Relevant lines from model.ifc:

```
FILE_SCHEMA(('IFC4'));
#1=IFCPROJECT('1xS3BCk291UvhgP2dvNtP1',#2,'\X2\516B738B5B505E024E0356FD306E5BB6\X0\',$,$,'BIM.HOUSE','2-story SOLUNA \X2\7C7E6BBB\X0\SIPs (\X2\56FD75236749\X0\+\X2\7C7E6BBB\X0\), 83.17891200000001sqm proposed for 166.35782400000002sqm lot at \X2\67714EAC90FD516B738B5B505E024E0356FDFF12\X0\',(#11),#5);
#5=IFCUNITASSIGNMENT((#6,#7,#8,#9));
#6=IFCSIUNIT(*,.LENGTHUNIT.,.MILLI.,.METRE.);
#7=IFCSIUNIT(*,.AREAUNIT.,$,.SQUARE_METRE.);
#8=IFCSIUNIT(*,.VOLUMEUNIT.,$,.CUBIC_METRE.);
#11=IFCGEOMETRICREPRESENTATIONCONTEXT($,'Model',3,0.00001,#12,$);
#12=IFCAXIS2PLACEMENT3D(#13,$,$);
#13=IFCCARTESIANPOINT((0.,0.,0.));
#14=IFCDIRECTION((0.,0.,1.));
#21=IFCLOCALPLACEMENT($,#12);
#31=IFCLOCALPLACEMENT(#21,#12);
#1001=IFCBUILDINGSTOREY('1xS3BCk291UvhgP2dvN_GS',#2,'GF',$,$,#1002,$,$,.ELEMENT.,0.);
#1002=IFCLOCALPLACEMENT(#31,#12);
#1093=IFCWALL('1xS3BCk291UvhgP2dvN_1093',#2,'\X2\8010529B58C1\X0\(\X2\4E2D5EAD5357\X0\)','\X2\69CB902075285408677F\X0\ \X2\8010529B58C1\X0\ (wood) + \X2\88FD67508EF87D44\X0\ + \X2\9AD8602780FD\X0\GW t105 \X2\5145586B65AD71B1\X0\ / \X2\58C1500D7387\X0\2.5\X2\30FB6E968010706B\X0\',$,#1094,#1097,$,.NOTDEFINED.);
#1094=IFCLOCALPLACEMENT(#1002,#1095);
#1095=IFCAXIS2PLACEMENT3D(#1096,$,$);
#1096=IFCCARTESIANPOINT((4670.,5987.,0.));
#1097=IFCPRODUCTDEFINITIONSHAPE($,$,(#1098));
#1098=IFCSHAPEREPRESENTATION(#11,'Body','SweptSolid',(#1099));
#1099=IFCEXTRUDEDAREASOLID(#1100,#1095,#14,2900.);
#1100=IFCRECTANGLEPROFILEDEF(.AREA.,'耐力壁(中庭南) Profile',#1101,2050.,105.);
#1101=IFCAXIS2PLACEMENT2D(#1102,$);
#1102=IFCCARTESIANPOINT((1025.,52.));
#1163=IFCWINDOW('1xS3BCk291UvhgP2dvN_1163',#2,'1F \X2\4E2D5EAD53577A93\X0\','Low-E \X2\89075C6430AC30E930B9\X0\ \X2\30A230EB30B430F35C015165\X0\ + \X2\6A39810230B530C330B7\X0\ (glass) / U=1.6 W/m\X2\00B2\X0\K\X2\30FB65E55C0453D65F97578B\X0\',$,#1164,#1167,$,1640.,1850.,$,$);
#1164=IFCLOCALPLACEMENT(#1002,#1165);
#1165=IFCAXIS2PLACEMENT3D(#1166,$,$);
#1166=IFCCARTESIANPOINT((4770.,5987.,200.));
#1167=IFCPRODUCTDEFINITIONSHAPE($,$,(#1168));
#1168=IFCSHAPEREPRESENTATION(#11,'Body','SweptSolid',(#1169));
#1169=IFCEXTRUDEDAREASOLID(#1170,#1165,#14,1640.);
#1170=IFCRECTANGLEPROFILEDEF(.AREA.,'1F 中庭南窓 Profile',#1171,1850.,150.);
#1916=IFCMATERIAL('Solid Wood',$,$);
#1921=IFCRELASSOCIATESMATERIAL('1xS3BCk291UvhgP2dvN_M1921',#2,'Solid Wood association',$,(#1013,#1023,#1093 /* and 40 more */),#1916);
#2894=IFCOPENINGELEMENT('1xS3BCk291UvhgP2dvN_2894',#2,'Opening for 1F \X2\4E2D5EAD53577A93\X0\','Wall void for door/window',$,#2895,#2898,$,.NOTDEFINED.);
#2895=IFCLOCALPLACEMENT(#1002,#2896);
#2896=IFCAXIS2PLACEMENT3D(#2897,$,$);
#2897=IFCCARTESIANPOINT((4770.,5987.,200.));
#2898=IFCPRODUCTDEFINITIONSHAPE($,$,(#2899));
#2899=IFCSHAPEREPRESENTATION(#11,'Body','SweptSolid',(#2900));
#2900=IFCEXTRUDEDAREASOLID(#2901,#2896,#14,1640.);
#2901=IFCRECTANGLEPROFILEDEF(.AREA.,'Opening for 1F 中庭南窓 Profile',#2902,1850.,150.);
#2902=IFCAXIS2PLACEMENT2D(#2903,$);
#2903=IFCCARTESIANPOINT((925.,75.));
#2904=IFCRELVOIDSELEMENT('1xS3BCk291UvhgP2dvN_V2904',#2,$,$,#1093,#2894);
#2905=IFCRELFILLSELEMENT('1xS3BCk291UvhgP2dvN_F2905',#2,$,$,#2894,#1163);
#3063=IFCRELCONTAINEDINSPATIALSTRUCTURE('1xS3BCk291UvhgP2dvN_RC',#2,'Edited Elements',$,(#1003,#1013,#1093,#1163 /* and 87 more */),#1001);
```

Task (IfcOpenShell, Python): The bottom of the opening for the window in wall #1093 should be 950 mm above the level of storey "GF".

```python
import numpy as np
import ifcopenshell
import ifcopenshell.api.geometry
import ifcopenshell.geom
import ifcopenshell.util.element
import ifcopenshell.util.placement
import ifcopenshell.util.shape
import ifcopenshell.util.unit

model = ifcopenshell.open("model.ifc")
unit_scale = ifcopenshell.util.unit.calculate_unit_scale(model)

window = model.by_guid("1xS3BCk291UvhgP2dvN_1163")
opening = window.FillsVoids[0].RelatingOpeningElement
storey = ifcopenshell.util.element.get_container(window, ifc_class="IfcBuildingStorey")
level = ifcopenshell.util.placement.get_local_placement(storey.ObjectPlacement)[2, 3]

# The opening's origin need not be at the sill, so measure its lowest point.
shape = ifcopenshell.geom.create_shape(ifcopenshell.geom.settings(), opening)
bottom = ifcopenshell.util.shape.get_shape_bottom_elevation(shape, shape.geometry) / unit_scale
dz = level + 0.95 / unit_scale - bottom

shift = np.array([0.0, 0.0, dz])
# The window is not placed relative to its opening, so move both.
for product in (opening, window):
    matrix = ifcopenshell.util.placement.get_local_placement(product.ObjectPlacement)
    matrix[:3, 3] += shift
    ifcopenshell.api.geometry.edit_object_placement(model, product=product, matrix=matrix, is_si=False)

print(f"moved by {dz * unit_scale:+.3f} m")

model.write("model_edited.ifc")
```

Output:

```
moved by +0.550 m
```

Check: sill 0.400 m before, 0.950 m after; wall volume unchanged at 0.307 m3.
